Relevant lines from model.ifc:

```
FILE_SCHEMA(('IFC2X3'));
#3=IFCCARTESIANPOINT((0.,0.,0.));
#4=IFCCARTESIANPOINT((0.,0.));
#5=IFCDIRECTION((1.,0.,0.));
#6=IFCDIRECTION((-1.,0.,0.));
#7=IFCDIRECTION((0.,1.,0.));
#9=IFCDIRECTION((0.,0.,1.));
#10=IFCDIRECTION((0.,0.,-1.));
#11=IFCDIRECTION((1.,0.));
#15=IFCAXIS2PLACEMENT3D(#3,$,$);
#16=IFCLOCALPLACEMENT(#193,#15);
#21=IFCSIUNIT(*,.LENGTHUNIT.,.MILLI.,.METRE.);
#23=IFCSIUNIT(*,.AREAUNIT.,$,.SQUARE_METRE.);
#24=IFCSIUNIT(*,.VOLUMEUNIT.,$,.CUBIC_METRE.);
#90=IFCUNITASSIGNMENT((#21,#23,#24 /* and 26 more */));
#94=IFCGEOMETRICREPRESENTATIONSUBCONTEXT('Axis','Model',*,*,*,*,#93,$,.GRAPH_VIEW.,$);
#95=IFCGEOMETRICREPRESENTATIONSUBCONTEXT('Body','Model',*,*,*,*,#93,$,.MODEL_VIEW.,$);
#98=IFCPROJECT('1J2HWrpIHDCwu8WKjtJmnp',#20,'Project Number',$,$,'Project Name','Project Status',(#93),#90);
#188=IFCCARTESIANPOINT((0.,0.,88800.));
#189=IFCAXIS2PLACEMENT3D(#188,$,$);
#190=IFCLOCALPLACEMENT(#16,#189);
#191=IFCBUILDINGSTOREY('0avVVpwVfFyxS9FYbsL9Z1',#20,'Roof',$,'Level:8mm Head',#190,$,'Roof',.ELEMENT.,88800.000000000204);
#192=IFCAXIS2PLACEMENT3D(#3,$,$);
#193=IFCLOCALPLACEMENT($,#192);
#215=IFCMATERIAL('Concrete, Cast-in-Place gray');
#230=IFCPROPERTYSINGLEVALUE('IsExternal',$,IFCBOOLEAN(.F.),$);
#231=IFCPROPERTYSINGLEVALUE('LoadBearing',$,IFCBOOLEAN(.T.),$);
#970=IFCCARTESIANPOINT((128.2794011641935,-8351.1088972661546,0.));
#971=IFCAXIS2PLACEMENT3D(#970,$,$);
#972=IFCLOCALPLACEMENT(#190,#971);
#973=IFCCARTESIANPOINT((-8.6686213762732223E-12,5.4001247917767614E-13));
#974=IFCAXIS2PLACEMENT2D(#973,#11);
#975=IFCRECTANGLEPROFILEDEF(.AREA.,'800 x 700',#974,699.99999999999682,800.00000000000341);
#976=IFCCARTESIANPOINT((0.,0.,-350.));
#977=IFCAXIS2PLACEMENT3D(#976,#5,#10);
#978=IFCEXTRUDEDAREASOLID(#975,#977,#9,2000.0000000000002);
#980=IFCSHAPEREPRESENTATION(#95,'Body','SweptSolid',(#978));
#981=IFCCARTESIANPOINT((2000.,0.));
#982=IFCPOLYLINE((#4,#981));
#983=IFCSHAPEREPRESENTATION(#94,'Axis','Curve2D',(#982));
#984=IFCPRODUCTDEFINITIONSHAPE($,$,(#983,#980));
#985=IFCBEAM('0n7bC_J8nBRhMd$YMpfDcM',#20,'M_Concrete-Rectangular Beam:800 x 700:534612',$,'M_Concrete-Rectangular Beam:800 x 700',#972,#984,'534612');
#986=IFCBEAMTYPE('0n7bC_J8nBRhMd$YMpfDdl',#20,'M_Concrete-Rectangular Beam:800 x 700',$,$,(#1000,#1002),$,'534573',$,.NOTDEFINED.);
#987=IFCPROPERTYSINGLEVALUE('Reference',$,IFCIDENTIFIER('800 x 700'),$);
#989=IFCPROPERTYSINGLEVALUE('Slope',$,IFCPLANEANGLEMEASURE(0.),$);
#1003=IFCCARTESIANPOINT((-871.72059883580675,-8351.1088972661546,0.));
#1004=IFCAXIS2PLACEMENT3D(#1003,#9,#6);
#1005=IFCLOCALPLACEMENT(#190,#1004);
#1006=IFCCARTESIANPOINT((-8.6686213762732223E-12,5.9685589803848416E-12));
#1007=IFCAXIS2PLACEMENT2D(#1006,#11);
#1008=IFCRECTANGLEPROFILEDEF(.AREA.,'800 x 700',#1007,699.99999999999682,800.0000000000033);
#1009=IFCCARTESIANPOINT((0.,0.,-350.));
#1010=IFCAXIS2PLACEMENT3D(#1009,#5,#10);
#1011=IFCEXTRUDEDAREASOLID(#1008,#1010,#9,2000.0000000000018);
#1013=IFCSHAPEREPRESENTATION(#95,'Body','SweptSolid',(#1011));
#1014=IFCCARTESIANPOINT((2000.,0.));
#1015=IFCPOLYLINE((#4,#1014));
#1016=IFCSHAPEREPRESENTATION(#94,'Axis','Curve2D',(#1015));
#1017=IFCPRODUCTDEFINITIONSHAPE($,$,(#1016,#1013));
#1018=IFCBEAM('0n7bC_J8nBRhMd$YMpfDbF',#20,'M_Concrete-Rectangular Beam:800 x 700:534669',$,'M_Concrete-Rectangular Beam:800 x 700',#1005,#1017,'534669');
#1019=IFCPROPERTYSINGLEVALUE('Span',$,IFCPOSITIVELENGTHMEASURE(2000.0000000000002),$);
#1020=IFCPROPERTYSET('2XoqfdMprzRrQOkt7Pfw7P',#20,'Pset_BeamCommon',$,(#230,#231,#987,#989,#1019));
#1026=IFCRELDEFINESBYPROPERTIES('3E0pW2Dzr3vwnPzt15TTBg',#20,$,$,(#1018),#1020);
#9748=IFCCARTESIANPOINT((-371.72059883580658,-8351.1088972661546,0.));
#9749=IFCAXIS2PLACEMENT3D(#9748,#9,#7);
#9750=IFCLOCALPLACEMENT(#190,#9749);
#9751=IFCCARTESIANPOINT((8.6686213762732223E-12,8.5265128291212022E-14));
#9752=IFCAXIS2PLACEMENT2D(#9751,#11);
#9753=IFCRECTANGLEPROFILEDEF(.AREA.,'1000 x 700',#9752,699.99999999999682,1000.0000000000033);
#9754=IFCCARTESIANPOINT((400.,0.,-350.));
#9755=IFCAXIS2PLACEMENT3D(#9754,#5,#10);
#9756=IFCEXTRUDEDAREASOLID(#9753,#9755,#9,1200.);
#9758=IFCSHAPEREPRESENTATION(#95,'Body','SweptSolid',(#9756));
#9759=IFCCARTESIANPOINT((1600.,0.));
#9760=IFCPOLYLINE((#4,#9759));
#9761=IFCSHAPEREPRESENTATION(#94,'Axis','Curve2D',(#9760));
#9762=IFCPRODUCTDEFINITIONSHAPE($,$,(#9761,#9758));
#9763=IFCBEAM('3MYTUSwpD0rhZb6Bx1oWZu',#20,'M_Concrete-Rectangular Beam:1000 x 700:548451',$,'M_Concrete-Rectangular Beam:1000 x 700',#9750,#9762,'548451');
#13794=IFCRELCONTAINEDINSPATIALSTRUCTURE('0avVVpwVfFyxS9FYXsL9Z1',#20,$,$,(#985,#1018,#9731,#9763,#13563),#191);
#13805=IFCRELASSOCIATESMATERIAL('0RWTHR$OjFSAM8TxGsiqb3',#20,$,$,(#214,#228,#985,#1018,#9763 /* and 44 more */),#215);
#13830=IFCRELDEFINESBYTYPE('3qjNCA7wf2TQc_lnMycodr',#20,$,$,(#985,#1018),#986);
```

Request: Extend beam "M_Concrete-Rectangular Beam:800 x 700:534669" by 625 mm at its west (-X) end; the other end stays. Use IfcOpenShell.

```python
import numpy as np
import ifcopenshell
import ifcopenshell.api.pset
import ifcopenshell.util.element
import ifcopenshell.util.representation

model = ifcopenshell.open("model.ifc")

member = model.by_guid("0n7bC_J8nBRhMd$YMpfDbF")
change = 625.0

# The extrusion runs towards the end named, so only its depth changes.
body = ifcopenshell.util.representation.get_representation(member, "Model", "Body")
solid = body.Items[0]
old_length = solid.Depth
solid.Depth += change

# Move the axis end point with it.
axis = next(r for r in member.Representation.Representations if r.RepresentationIdentifier == "Axis").Items[0]
start, end = (np.array(p.Coordinates) for p in axis.Points)
end = end + (end - start) / np.linalg.norm(end - start) * change
point = model.createIfcCartesianPoint(end.tolist())
axis.Points = [axis.Points[0], point]

# Update the stored length and volume.
pset = model.by_id(ifcopenshell.util.element.get_pset(member, "Pset_BeamCommon", should_inherit=False)["id"])
ifcopenshell.api.pset.edit_pset(model, pset=pset, properties={
    "Span": model.create_entity("IfcPositiveLengthMeasure", solid.Depth),
})

print(f"length {old_length:g} -> {solid.Depth:g}")

model.write("model_edited.ifc")
```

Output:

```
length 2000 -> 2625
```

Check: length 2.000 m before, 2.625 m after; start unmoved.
